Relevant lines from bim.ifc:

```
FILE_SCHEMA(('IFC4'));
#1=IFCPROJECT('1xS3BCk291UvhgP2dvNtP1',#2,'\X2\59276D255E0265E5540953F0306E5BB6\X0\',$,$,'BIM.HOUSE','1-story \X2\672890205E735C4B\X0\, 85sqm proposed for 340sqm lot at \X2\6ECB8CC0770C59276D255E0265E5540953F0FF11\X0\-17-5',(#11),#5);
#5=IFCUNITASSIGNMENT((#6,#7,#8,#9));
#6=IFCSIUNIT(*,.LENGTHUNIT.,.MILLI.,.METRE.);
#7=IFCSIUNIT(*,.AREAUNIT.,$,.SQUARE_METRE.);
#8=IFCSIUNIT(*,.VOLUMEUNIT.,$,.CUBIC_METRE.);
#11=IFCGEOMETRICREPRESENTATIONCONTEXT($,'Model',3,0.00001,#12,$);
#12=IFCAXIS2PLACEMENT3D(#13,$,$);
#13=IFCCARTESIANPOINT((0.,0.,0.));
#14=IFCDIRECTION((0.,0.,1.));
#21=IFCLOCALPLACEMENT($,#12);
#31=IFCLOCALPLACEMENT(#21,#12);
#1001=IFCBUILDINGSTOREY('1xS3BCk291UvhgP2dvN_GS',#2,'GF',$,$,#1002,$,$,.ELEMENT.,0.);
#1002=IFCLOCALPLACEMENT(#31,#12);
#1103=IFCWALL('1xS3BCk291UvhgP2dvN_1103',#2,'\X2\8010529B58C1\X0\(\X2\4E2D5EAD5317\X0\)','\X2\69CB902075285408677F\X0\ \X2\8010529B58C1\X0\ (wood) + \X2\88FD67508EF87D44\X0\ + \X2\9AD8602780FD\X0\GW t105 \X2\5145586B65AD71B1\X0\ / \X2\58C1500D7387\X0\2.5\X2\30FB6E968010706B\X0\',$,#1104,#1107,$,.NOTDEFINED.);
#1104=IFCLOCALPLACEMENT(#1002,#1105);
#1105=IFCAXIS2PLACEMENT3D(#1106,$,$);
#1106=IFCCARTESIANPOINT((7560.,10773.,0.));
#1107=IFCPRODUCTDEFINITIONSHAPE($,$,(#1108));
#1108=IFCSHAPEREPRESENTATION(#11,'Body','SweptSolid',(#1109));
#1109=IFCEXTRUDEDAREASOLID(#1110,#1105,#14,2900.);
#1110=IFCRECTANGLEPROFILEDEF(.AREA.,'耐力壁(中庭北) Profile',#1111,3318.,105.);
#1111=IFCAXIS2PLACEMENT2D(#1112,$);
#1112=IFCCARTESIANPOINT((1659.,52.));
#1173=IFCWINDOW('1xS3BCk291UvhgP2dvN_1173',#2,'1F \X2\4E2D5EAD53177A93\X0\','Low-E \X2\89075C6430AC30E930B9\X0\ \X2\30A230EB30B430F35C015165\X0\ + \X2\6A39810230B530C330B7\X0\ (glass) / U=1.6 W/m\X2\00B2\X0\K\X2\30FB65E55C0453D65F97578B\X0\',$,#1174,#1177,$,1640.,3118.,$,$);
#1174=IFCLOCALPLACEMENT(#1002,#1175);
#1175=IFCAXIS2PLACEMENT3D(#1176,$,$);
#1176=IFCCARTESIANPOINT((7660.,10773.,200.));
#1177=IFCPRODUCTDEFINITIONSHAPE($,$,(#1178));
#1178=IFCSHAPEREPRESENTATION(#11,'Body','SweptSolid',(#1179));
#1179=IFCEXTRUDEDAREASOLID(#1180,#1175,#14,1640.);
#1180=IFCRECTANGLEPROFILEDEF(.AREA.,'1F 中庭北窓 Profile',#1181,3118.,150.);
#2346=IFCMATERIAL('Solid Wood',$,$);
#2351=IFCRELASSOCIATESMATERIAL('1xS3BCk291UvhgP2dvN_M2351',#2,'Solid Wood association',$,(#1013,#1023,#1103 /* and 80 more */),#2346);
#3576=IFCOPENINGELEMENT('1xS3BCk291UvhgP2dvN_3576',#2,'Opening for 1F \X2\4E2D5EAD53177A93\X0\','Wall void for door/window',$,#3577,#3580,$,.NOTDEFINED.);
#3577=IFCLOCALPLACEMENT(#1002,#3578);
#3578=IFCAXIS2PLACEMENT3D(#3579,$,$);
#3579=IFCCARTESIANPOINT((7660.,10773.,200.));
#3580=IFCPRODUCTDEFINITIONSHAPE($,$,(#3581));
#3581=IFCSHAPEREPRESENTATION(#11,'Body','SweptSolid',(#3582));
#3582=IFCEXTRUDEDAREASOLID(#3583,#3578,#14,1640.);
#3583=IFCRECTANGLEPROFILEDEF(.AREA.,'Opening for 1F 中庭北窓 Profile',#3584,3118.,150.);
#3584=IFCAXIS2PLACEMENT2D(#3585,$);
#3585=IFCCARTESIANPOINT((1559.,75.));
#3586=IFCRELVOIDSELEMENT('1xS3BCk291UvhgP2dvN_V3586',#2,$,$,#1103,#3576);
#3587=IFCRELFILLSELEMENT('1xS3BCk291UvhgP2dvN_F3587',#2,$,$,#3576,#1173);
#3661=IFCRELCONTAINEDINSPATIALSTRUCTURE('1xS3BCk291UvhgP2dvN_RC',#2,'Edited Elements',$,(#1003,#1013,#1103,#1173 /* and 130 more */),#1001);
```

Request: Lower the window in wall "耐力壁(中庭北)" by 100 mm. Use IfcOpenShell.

```python
import numpy as np
import ifcopenshell
import ifcopenshell.api.geometry
import ifcopenshell.util.placement
import ifcopenshell.util.unit

model = ifcopenshell.open("bim.ifc")
unit_scale = ifcopenshell.util.unit.calculate_unit_scale(model)

window = model.by_guid("1xS3BCk291UvhgP2dvN_1173")
opening = window.FillsVoids[0].RelatingOpeningElement
dz = -0.1 / unit_scale

shift = np.array([0.0, 0.0, dz])
# The window is not placed relative to its opening, so move both.
for product in (opening, window):
    matrix = ifcopenshell.util.placement.get_local_placement(product.ObjectPlacement)
    matrix[:3, 3] += shift
    ifcopenshell.api.geometry.edit_object_placement(model, product=product, matrix=matrix, is_si=False)

print(f"moved by {dz * unit_scale:+.3f} m")

model.write("bim-out.ifc")
```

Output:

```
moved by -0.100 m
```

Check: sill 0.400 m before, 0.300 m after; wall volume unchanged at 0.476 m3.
